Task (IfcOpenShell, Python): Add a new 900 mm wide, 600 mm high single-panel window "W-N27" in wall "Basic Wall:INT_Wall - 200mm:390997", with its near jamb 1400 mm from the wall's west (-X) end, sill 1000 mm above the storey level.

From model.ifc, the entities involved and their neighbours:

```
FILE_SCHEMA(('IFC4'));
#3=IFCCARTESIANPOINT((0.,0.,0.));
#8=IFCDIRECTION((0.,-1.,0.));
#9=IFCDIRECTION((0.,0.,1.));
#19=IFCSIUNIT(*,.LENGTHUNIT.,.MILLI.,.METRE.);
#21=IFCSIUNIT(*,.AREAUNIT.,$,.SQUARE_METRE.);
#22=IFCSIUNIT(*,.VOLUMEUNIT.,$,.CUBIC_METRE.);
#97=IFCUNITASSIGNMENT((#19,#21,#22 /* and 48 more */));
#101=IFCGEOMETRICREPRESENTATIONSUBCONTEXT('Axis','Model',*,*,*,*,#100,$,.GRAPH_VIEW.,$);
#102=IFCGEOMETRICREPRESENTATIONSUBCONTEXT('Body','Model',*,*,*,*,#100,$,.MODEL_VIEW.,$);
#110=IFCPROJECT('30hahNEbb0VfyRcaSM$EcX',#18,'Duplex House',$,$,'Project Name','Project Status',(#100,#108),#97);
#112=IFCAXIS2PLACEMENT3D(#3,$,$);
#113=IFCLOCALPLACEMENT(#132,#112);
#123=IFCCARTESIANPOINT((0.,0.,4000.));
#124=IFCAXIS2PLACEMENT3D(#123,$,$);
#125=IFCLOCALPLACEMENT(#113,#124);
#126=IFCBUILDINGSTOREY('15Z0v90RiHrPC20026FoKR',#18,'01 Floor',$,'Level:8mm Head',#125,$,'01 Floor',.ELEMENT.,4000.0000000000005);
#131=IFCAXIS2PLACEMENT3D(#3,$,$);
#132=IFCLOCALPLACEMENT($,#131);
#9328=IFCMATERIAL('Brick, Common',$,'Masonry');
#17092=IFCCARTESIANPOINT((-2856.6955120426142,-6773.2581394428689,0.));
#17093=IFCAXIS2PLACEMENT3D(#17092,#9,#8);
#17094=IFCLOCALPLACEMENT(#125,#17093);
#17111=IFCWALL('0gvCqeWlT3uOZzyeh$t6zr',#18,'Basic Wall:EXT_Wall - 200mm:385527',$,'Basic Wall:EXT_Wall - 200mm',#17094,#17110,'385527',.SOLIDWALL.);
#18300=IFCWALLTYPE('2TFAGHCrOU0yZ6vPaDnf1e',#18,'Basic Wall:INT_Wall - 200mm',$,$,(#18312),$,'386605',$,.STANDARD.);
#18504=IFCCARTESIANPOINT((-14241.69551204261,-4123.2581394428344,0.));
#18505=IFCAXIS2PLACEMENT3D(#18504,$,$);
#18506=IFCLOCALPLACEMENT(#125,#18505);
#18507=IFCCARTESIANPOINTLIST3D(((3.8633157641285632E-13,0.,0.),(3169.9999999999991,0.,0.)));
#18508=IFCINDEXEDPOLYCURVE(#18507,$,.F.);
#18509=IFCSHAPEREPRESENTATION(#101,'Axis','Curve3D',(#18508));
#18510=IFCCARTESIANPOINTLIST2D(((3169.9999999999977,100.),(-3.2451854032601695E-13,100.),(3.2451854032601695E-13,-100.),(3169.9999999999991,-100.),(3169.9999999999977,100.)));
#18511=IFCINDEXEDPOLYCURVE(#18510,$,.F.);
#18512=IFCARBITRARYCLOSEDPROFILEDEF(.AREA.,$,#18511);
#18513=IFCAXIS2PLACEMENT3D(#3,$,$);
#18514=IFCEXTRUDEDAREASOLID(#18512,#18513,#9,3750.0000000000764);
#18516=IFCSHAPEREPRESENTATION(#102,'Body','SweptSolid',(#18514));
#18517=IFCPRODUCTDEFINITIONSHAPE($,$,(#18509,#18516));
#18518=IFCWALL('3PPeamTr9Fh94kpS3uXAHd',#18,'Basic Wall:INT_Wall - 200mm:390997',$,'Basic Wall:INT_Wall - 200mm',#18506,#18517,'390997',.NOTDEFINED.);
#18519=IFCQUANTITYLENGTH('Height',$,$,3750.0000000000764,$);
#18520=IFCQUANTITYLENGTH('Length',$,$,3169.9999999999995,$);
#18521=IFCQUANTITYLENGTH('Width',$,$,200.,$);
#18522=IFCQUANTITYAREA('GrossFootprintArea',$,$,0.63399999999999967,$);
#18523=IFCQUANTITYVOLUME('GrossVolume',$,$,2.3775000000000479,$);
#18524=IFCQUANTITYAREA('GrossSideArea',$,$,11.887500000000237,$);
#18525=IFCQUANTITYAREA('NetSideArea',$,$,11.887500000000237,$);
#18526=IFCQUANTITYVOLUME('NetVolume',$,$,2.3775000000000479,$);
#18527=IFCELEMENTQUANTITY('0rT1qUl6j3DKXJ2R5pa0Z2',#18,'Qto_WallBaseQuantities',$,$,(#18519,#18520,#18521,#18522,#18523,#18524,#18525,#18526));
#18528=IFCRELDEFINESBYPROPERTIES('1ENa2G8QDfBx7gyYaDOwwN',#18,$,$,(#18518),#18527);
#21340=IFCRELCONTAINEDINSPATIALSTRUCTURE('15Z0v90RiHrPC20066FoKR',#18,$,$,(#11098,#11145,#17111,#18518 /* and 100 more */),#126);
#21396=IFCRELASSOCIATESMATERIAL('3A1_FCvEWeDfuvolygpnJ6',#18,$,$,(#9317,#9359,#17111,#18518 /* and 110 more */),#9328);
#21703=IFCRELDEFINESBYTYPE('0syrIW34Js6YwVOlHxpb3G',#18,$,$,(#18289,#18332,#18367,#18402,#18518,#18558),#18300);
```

```python
import numpy as np
import ifcopenshell
import ifcopenshell.api.feature
import ifcopenshell.api.geometry
import ifcopenshell.api.pset
import ifcopenshell.api.root
import ifcopenshell.api.spatial
import ifcopenshell.geom
import ifcopenshell.util.element
import ifcopenshell.util.placement
import ifcopenshell.util.representation
import ifcopenshell.util.shape
import ifcopenshell.util.unit

model = ifcopenshell.open("model.ifc")
unit_scale = ifcopenshell.util.unit.calculate_unit_scale(model)
area_scale = ifcopenshell.util.unit.calculate_unit_scale(model, "AREAUNIT")
volume_scale = ifcopenshell.util.unit.calculate_unit_scale(model, "VOLUMEUNIT")
settings = ifcopenshell.geom.settings()


def volume(element):
    """Net volume in cubic metres, openings subtracted."""
    shape = ifcopenshell.geom.create_shape(settings, element)
    return ifcopenshell.util.shape.get_volume(shape.geometry)


wall = model.by_id(18518)
storey = ifcopenshell.util.element.get_container(wall, ifc_class="IfcBuildingStorey")
context = ifcopenshell.util.representation.get_context(model, "Model", "Body", "MODEL_VIEW")
before = volume(wall)

width, height, from_end, sill = 0.9, 0.6, 1.4, 1  # metres

# The wall runs along its own X axis, and the end named is its -X end.
wall_shape = ifcopenshell.geom.create_shape(settings, wall)
x, y, z = ifcopenshell.util.shape.get_vertices(wall_shape.geometry).T
start = x.min() + from_end
face, thickness = float(y.min()), float(y.max() - y.min())
wall_matrix = ifcopenshell.util.placement.get_local_placement(wall.ObjectPlacement)
level = ifcopenshell.util.placement.get_local_placement(storey.ObjectPlacement)[2, 3]


def in_wall(x, y):
    """Placement at x, y metres in the wall's axes, at sill height."""
    matrix = wall_matrix.copy()
    matrix[:, 3] = wall_matrix @ np.array([x / unit_scale, y / unit_scale, 0.0, 1.0])
    matrix[2, 3] = level + sill / unit_scale
    return matrix


# Opening: a box that overshoots both wall faces by 50 mm.
opening = ifcopenshell.api.root.create_entity(model, ifc_class="IfcOpeningElement", predefined_type="OPENING")
box = ifcopenshell.api.geometry.add_wall_representation(
    model, context=context, length=width, height=height, thickness=thickness + 0.1
)
ifcopenshell.api.geometry.assign_representation(model, product=opening, representation=box)
ifcopenshell.api.geometry.edit_object_placement(model, product=opening, matrix=in_wall(start, face - 0.05), is_si=False)
ifcopenshell.api.feature.add_feature(model, feature=opening, element=wall)

window = ifcopenshell.api.root.create_entity(model, ifc_class="IfcWindow", name="W-N27", predefined_type="WINDOW")
window.OverallWidth, window.OverallHeight = width / unit_scale, height / unit_scale
window.PartitioningType = "SINGLE_PANEL"
body = ifcopenshell.api.geometry.add_window_representation(
    model,
    context=context,
    overall_width=window.OverallWidth,
    overall_height=window.OverallHeight,
    partition_type="SINGLE_PANEL",
)
ifcopenshell.api.geometry.assign_representation(model, product=window, representation=body)
ifcopenshell.api.spatial.assign_container(model, products=[window], relating_structure=storey)
ifcopenshell.api.feature.add_filling(model, opening=opening, element=window)

# Centre the window in the wall's thickness.
ifcopenshell.api.geometry.edit_object_placement(model, product=window, matrix=in_wall(start, face), is_si=False)
window_shape = ifcopenshell.geom.create_shape(settings, window)
depth = ifcopenshell.util.shape.get_vertices(window_shape.geometry)[:, 1]
offset = face + thickness / 2 - (depth.min() + depth.max()) / 2
ifcopenshell.api.geometry.edit_object_placement(model, product=window, matrix=in_wall(start, offset), is_si=False)

after = volume(wall)

# Update the wall's stored quantities.
qto = model.by_id(ifcopenshell.util.element.get_pset(wall, "Qto_WallBaseQuantities", should_inherit=False)["id"])
ifcopenshell.api.pset.edit_qto(model, qto=qto, properties={
    "NetSideArea": after / thickness / area_scale,
    "NetVolume": after / volume_scale,
})

print(f"wall volume {before:.3f} -> {after:.3f} m3")

model.write("model_edited.ifc")
```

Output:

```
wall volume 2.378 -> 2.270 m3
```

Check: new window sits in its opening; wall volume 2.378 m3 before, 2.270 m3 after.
